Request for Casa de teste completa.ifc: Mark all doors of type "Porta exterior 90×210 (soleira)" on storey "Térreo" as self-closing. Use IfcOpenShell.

First a look at what the model holds.

```python
import ifcopenshell
import ifcopenshell.util.element

model = ifcopenshell.open("Casa de teste completa.ifc")
print(model.schema)
storey = next(s for s in model.by_type("IfcBuildingStorey") if s.Name == "Térreo")
doors = [e for e in ifcopenshell.util.element.get_decomposition(storey) if e.is_a("IfcDoor")]
seen = {}
for e in doors:
    element_type = ifcopenshell.util.element.get_type(e)
    key = (element_type.Name if element_type != e and element_type else None, ifcopenshell.util.element.get_pset(e, "Pset_DoorCommon", "SelfClosing"))
    seen[key] = seen.get(key, 0) + 1
for (name, value), count in sorted(seen.items(), key=str):
    print(count, "x", name, "|", value)
```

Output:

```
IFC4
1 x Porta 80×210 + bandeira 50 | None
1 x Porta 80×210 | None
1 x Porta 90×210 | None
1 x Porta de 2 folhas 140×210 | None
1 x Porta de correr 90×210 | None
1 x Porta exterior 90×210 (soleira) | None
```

```python
import ifcopenshell
import ifcopenshell.api.pset
import ifcopenshell.util.element

model = ifcopenshell.open("Casa de teste completa.ifc")

storey = next(s for s in model.by_type("IfcBuildingStorey") if s.Name == "Térreo")
doors = [e for e in ifcopenshell.util.element.get_decomposition(storey) if e.is_a("IfcDoor")]

count = 0
for e in doors:
    element_type = ifcopenshell.util.element.get_type(e)
    if element_type in (None, e) or element_type.Name != "Porta exterior 90×210 (soleira)":
        continue
    # add_pset returns the element's existing set when there is one.
    pset = ifcopenshell.api.pset.add_pset(model, product=e, name="Pset_DoorCommon")
    ifcopenshell.api.pset.edit_pset(model, pset=pset, properties={"SelfClosing": True})
    count += 1

print(count, "doors updated")

model.write("Casa de teste completa-out.ifc")
```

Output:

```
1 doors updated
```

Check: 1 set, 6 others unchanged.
